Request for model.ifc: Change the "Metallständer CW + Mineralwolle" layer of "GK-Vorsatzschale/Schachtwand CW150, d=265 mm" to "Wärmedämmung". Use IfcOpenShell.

First a look at what the model holds.

```python
import ifcopenshell
import ifcopenshell.util.element

model = ifcopenshell.open("model.ifc")
print(model.schema)
for layer_set in model.by_type("IfcMaterialLayerSet"):
    if layer_set.LayerSetName == "GK-Vorsatzschale/Schachtwand CW150, d=265 mm":
        for layer in layer_set.MaterialLayers:
            print(layer.id(), layer.Material and layer.Material.Name, layer.LayerThickness, sep=" | ")
        print(len(ifcopenshell.util.element.get_elements_by_material(model, layer_set)), "elements and types use it")
print(sorted(m.Name for m in model.by_type("IfcMaterial") if m.Name)[:60])
```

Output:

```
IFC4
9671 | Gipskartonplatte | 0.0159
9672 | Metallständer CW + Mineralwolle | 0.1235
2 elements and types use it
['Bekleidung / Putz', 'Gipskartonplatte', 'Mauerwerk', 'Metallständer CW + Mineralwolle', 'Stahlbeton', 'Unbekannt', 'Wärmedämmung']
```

```python
import ifcopenshell
import ifcopenshell.api.material

model = ifcopenshell.open("model.ifc")

layer_set = next(s for s in model.by_type("IfcMaterialLayerSet") if s.LayerSetName == "GK-Vorsatzschale/Schachtwand CW150, d=265 mm")
layer = next(l for l in layer_set.MaterialLayers if l.Material and l.Material.Name == "Metallständer CW + Mineralwolle")
material = next(m for m in model.by_type("IfcMaterial") if m.Name == "Wärmedämmung")

# Point this one layer at the other material; renaming the old one would change it everywhere.
ifcopenshell.api.material.edit_layer(model, layer=layer, attributes={"Name": material.Name}, material=material)

print([l.Material.Name if l.Material else None for l in layer_set.MaterialLayers])

model.write("model_edited.ifc")
```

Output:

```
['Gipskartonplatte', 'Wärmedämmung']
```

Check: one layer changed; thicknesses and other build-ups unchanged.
